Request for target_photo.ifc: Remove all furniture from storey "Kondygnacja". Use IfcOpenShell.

First a look at what the model holds.

```python
import ifcopenshell
import ifcopenshell.util.element

model = ifcopenshell.open("target_photo.ifc")
print(model.schema)
storey = next(s for s in model.by_type("IfcBuildingStorey") if s.Name == "Kondygnacja")
furniture = [e for e in ifcopenshell.util.element.get_decomposition(storey) if e.is_a("IfcFurnishingElement")]
seen = {}
for e in furniture:
    element_type = ifcopenshell.util.element.get_type(e)
    name = element_type.Name if element_type not in (None, e) else None
    seen[name] = seen.get(name, 0) + 1
for name, count in sorted(seen.items(), key=str):
    print(count, "x", name)
```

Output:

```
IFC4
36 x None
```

```python
import ifcopenshell
import ifcopenshell.api.root
import ifcopenshell.util.element

model = ifcopenshell.open("target_photo.ifc")

storey = next(s for s in model.by_type("IfcBuildingStorey") if s.Name == "Kondygnacja")
furniture = [e for e in ifcopenshell.util.element.get_decomposition(storey) if e.is_a("IfcFurnishingElement")]

for e in furniture:
    ifcopenshell.api.root.remove_product(model, product=e)
print(len(furniture), "removed")

model.write("target_photo_v2.ifc")
```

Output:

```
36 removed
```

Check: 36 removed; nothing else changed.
